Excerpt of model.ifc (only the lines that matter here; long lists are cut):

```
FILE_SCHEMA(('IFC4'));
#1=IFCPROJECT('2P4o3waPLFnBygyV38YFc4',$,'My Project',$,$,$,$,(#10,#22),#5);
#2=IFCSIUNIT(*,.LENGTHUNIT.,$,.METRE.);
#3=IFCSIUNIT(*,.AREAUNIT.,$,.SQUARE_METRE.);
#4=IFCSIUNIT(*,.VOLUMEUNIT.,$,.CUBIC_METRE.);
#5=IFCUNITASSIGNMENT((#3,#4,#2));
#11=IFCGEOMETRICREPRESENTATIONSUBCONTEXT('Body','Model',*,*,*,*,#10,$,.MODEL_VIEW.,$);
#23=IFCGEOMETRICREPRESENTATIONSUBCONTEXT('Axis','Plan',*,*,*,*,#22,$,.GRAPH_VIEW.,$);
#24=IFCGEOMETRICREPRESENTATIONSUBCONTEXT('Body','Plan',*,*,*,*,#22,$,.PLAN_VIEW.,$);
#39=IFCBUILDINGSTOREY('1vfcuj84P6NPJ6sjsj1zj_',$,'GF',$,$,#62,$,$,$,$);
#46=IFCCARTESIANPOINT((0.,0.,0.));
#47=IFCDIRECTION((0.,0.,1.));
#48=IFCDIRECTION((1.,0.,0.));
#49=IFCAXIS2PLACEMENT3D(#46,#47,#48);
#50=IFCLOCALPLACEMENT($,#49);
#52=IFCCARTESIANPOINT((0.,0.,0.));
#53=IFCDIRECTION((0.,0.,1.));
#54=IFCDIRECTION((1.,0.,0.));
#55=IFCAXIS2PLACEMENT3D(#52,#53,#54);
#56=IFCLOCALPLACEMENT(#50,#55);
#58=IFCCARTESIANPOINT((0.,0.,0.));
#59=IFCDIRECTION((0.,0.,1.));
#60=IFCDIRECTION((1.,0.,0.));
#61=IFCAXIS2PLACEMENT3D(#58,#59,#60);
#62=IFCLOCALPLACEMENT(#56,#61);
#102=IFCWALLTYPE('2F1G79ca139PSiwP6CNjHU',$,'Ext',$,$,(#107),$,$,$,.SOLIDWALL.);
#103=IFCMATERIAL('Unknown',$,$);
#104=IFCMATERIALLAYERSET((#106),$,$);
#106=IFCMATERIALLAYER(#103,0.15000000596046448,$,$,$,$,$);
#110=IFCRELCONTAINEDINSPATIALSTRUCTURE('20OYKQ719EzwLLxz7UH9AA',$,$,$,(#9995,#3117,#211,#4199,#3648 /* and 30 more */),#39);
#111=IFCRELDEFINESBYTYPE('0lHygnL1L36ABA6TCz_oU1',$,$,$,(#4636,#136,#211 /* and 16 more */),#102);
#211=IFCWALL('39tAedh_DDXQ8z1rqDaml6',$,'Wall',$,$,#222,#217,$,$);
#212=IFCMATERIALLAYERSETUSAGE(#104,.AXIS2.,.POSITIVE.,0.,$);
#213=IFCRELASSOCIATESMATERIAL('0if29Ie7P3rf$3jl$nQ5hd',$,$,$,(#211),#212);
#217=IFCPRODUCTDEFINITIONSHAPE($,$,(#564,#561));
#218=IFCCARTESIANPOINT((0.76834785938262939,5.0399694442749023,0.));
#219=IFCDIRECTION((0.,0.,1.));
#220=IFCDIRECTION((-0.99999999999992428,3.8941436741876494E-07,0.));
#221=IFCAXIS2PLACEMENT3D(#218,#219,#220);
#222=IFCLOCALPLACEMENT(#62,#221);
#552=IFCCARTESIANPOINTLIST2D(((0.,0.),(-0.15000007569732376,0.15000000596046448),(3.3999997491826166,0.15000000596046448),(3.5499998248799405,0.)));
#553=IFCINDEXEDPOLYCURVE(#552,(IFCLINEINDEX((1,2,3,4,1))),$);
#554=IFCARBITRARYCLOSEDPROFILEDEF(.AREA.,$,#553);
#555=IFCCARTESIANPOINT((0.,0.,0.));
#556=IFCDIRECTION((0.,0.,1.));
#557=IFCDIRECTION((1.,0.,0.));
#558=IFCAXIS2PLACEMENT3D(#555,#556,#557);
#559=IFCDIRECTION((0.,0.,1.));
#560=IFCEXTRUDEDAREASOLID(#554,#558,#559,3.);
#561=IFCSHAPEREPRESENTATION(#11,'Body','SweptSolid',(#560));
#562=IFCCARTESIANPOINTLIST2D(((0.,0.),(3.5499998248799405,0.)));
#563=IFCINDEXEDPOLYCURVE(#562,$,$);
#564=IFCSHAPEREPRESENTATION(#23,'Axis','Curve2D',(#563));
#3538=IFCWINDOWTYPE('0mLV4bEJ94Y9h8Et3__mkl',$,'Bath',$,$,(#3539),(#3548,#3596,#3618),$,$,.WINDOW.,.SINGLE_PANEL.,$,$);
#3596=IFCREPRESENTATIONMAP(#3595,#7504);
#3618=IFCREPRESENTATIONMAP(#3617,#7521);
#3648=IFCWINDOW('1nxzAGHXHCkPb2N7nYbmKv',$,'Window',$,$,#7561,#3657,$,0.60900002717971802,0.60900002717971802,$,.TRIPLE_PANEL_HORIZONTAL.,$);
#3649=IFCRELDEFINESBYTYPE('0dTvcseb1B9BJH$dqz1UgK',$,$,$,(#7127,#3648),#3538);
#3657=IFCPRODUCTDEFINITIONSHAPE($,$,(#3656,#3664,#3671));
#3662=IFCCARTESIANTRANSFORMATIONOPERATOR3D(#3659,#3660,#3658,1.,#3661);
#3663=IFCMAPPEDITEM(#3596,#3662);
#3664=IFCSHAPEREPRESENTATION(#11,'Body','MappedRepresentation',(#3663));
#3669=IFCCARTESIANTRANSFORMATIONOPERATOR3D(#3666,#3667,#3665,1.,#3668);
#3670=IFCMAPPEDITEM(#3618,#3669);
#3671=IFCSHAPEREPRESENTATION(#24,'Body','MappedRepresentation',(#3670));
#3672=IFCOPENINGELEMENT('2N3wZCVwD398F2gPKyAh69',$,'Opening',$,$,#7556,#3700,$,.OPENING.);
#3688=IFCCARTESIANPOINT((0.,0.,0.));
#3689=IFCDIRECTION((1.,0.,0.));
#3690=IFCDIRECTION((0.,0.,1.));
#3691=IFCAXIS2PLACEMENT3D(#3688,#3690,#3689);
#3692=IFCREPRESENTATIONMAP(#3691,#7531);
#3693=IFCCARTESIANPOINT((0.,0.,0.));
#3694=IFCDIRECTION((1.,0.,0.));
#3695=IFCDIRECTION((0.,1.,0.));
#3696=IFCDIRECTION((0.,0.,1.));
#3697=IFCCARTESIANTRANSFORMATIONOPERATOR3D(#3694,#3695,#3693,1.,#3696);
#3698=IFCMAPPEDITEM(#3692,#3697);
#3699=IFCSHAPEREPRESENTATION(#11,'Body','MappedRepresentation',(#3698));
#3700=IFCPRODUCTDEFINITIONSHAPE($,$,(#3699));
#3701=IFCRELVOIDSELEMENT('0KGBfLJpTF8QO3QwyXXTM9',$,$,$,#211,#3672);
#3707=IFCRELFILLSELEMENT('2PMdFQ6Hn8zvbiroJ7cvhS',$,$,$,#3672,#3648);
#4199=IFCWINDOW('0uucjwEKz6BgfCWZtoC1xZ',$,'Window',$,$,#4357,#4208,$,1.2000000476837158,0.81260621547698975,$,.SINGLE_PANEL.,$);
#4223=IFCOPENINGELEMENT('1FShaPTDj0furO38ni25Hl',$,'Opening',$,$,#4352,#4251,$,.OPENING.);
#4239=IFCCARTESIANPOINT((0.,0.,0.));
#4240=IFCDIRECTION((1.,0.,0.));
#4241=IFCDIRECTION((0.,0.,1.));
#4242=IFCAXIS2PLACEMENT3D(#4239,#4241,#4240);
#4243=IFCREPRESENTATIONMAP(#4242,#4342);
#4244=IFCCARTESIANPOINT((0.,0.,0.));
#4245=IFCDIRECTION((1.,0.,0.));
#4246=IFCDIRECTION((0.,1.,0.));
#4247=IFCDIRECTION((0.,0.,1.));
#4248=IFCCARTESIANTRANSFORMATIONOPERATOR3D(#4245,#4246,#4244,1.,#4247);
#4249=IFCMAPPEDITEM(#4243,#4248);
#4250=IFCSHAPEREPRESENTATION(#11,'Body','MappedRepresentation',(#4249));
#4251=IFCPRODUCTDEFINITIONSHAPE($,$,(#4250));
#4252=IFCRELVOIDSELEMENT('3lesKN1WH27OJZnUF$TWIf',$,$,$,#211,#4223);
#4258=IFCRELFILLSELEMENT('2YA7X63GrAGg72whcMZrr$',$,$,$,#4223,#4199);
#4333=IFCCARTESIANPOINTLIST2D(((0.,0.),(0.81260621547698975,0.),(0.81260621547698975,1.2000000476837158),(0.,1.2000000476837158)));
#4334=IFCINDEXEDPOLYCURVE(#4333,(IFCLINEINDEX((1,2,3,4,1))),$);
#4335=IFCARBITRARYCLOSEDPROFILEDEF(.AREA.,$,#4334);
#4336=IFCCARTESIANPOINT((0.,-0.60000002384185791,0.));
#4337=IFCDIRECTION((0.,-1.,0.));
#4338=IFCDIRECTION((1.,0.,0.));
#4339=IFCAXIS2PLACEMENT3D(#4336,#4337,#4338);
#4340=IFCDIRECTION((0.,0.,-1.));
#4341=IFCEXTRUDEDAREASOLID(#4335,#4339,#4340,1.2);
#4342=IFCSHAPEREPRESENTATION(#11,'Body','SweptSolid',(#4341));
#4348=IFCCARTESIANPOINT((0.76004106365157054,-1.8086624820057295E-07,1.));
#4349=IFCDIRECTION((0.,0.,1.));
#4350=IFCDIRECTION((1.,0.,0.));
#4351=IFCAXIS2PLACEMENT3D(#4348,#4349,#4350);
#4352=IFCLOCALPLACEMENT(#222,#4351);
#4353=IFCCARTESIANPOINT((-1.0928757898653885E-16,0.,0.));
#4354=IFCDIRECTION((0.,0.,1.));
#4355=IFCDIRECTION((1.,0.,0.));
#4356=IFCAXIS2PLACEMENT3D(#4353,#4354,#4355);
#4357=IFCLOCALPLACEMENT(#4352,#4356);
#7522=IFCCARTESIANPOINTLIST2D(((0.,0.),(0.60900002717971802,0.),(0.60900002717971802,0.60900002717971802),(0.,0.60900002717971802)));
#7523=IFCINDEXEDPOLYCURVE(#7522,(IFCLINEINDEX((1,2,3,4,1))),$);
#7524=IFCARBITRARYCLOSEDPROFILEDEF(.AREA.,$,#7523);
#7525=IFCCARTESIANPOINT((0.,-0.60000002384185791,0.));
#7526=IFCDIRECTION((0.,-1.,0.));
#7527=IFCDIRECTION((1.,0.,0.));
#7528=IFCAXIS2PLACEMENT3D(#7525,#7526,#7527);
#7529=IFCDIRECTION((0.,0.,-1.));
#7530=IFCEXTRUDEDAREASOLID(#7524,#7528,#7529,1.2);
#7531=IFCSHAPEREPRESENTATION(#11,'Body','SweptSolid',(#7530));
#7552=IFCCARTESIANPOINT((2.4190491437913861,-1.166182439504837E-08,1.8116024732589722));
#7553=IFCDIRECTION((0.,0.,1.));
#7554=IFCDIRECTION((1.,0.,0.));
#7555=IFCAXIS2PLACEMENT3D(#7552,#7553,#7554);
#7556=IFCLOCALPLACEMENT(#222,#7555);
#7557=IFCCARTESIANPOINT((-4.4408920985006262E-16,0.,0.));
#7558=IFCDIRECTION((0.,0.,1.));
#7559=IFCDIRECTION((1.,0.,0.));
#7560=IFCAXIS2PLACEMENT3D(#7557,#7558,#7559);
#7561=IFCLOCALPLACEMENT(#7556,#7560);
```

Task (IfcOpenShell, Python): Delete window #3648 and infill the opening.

```python
import ifcopenshell
import ifcopenshell.api.feature
import ifcopenshell.api.root
import ifcopenshell.geom
import ifcopenshell.util.shape

model = ifcopenshell.open("model.ifc")
settings = ifcopenshell.geom.settings()


def volume(element):
    """Net volume in cubic metres, openings subtracted."""
    shape = ifcopenshell.geom.create_shape(settings, element)
    return ifcopenshell.util.shape.get_volume(shape.geometry)


window = model.by_guid("1nxzAGHXHCkPb2N7nYbmKv")
opening = window.FillsVoids[0].RelatingOpeningElement
wall = opening.VoidsElements[0].RelatingBuildingElement
before = volume(wall)

ifcopenshell.api.root.remove_product(model, product=window)
ifcopenshell.api.feature.remove_feature(model, feature=opening)

after = volume(wall)

print(f"wall volume {before:.3f} -> {after:.3f} m3")

model.write("model_v2.ifc")
```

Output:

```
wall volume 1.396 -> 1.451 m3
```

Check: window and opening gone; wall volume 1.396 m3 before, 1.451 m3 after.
